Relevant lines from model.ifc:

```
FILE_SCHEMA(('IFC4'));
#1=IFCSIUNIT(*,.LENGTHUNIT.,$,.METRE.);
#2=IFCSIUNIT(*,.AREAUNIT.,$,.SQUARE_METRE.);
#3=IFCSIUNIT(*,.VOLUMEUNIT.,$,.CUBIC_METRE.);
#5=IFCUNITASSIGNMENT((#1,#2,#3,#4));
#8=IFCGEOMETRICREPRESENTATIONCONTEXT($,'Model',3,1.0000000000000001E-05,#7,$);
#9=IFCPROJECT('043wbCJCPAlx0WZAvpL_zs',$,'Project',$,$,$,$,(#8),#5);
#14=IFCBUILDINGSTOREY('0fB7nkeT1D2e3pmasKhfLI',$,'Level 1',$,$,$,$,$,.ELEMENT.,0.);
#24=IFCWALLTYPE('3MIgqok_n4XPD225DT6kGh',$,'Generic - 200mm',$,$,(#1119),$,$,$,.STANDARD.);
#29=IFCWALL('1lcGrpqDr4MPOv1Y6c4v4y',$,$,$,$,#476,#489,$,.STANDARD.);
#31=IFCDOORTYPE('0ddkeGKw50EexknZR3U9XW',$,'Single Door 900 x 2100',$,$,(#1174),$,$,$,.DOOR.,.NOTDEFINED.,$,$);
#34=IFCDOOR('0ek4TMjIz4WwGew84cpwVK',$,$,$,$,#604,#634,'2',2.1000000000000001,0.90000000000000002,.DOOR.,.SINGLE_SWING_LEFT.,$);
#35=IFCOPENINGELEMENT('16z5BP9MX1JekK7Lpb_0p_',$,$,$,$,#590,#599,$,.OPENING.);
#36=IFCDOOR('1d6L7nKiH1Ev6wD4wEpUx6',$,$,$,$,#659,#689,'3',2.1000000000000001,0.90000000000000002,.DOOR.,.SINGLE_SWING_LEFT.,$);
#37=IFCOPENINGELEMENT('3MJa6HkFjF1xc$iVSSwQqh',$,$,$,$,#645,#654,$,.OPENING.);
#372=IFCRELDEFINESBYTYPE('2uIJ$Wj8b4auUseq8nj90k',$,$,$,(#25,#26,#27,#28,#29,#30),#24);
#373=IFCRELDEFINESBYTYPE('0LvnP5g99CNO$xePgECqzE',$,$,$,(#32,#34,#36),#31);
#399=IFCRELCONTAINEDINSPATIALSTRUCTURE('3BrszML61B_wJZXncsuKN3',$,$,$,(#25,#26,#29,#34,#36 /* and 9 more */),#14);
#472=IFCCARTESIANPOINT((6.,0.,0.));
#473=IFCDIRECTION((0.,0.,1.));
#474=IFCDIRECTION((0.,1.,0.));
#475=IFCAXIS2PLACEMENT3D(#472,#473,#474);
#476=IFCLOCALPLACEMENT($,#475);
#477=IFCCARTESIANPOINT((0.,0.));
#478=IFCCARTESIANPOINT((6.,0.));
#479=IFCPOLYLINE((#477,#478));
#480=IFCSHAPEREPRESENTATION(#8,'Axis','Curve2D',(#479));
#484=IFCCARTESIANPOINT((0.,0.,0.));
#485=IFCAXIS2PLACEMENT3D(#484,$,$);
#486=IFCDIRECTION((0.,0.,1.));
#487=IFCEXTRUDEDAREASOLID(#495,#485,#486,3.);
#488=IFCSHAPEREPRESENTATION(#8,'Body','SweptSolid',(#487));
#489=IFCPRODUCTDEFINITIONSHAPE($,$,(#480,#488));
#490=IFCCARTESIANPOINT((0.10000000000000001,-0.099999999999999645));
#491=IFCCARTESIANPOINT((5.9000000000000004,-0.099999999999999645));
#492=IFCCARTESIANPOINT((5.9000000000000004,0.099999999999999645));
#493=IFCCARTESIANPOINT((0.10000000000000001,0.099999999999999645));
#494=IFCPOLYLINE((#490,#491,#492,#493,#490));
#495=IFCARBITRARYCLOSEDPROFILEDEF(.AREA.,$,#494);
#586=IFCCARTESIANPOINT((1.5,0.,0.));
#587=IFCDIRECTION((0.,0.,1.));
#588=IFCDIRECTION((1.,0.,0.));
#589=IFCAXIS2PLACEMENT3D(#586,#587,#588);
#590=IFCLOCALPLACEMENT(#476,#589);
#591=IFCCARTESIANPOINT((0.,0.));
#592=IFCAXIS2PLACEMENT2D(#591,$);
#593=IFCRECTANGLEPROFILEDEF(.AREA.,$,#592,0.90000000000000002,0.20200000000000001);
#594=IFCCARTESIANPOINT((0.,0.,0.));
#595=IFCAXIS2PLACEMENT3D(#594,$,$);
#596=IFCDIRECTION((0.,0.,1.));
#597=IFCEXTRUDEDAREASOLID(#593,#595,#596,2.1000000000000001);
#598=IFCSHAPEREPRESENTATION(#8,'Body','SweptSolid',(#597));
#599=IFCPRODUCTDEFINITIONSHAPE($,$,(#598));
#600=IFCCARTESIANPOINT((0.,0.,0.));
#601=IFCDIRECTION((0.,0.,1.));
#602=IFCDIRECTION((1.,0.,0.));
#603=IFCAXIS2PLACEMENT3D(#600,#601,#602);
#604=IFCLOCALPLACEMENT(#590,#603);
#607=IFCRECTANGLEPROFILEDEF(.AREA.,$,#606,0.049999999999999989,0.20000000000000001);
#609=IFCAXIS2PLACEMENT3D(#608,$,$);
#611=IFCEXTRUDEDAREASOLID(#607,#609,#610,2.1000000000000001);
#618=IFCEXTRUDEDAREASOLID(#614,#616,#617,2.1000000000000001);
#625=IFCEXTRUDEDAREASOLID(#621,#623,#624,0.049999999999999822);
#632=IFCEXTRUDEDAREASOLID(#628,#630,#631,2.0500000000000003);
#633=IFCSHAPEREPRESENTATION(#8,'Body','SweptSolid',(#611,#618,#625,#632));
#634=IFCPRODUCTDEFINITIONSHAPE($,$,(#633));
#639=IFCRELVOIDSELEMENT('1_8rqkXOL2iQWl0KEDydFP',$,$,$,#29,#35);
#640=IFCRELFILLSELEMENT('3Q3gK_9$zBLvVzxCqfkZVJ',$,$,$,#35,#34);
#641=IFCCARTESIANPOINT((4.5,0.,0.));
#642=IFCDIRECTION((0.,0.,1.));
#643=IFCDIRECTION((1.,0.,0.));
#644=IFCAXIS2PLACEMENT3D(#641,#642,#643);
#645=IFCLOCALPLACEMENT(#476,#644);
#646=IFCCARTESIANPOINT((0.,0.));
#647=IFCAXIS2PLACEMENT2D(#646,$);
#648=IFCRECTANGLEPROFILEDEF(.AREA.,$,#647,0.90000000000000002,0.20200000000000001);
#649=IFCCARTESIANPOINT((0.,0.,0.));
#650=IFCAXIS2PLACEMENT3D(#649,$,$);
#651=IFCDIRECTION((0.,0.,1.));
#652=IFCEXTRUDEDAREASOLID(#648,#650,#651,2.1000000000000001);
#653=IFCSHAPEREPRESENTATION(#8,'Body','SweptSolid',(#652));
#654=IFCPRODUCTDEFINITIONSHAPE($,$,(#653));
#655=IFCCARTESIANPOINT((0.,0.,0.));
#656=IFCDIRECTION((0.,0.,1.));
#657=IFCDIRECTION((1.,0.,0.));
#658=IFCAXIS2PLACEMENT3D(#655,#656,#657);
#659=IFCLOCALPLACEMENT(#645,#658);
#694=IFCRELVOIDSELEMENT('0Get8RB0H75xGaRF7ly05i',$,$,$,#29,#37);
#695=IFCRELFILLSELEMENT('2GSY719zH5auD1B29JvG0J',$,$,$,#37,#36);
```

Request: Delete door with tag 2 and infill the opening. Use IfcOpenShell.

```python
import ifcopenshell
import ifcopenshell.api.feature
import ifcopenshell.api.root
import ifcopenshell.geom
import ifcopenshell.util.shape

model = ifcopenshell.open("model.ifc")
settings = ifcopenshell.geom.settings()


def volume(element):
    """Net volume in cubic metres, openings subtracted."""
    shape = ifcopenshell.geom.create_shape(settings, element)
    return ifcopenshell.util.shape.get_volume(shape.geometry)


door = model.by_id(34)
opening = door.FillsVoids[0].RelatingOpeningElement
wall = opening.VoidsElements[0].RelatingBuildingElement
before = volume(wall)

ifcopenshell.api.root.remove_product(model, product=door)
ifcopenshell.api.feature.remove_feature(model, feature=opening)

after = volume(wall)

print(f"wall volume {before:.3f} -> {after:.3f} m3")

model.write("model_rev.ifc")
```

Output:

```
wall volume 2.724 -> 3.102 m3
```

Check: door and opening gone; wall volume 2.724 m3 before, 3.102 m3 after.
